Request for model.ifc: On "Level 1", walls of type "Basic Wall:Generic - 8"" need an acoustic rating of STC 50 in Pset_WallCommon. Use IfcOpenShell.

First a look at what the model holds.

```python
import ifcopenshell
import ifcopenshell.util.element

model = ifcopenshell.open("model.ifc")
print(model.schema)
storey = next(s for s in model.by_type("IfcBuildingStorey") if s.Name == "Level 1")
walls = [e for e in ifcopenshell.util.element.get_decomposition(storey) if e.is_a("IfcWall")]
seen = {}
for e in walls:
    element_type = ifcopenshell.util.element.get_type(e)
    key = (element_type.Name if element_type != e and element_type else None, ifcopenshell.util.element.get_pset(e, "Pset_WallCommon", "AcousticRating"))
    seen[key] = seen.get(key, 0) + 1
for (name, value), count in sorted(seen.items(), key=str):
    print(count, "x", name, "|", value)
```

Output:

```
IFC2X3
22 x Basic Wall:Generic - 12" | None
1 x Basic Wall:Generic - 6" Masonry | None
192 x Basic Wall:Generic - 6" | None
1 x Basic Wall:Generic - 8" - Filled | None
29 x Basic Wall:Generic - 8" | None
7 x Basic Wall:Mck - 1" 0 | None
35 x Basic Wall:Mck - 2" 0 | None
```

```python
import ifcopenshell
import ifcopenshell.api.pset
import ifcopenshell.util.element

model = ifcopenshell.open("model.ifc")

storey = next(s for s in model.by_type("IfcBuildingStorey") if s.Name == "Level 1")
walls = [e for e in ifcopenshell.util.element.get_decomposition(storey) if e.is_a("IfcWall")]

count = 0
for e in walls:
    element_type = ifcopenshell.util.element.get_type(e)
    if element_type in (None, e) or element_type.Name != 'Basic Wall:Generic - 8"':
        continue
    # add_pset returns the element's existing set when there is one.
    pset = ifcopenshell.api.pset.add_pset(model, product=e, name="Pset_WallCommon")
    ifcopenshell.api.pset.edit_pset(model, pset=pset, properties={"AcousticRating": "STC 50"})
    count += 1

print(count, "walls updated")

model.write("model_v2.ifc")
```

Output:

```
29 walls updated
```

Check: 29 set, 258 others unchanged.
